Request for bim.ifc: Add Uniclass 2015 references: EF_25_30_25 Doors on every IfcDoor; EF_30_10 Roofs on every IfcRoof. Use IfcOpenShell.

First a look at what the model holds.

```python
import ifcopenshell

model = ifcopenshell.open("bim.ifc")
print(model.schema)
print("classifications:", [c.Name for c in model.by_type("IfcClassification")])
for ifc_class in ("IfcDoor", "IfcRoof", "IfcStair", "IfcWall", "IfcWindow"):
    print(ifc_class, len(model.by_type(ifc_class)))
```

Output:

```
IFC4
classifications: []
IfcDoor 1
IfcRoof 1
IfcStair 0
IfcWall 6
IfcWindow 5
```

```python
import ifcopenshell
import ifcopenshell.api.classification

model = ifcopenshell.open("bim.ifc")

system = ifcopenshell.api.classification.add_classification(model, classification="Uniclass 2015")

codes = {
    "IfcDoor": ("EF_25_30_25", "Doors"),
    "IfcRoof": ("EF_30_10", "Roofs"),
}
for ifc_class, (code, name) in codes.items():
    products = model.by_type(ifc_class)
    ifcopenshell.api.classification.add_reference(
        model, products=products, classification=system, identification=code, name=name
    )
    print(code, len(products))

model.write("bim_v2.ifc")
```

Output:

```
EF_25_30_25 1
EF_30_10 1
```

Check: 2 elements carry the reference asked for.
